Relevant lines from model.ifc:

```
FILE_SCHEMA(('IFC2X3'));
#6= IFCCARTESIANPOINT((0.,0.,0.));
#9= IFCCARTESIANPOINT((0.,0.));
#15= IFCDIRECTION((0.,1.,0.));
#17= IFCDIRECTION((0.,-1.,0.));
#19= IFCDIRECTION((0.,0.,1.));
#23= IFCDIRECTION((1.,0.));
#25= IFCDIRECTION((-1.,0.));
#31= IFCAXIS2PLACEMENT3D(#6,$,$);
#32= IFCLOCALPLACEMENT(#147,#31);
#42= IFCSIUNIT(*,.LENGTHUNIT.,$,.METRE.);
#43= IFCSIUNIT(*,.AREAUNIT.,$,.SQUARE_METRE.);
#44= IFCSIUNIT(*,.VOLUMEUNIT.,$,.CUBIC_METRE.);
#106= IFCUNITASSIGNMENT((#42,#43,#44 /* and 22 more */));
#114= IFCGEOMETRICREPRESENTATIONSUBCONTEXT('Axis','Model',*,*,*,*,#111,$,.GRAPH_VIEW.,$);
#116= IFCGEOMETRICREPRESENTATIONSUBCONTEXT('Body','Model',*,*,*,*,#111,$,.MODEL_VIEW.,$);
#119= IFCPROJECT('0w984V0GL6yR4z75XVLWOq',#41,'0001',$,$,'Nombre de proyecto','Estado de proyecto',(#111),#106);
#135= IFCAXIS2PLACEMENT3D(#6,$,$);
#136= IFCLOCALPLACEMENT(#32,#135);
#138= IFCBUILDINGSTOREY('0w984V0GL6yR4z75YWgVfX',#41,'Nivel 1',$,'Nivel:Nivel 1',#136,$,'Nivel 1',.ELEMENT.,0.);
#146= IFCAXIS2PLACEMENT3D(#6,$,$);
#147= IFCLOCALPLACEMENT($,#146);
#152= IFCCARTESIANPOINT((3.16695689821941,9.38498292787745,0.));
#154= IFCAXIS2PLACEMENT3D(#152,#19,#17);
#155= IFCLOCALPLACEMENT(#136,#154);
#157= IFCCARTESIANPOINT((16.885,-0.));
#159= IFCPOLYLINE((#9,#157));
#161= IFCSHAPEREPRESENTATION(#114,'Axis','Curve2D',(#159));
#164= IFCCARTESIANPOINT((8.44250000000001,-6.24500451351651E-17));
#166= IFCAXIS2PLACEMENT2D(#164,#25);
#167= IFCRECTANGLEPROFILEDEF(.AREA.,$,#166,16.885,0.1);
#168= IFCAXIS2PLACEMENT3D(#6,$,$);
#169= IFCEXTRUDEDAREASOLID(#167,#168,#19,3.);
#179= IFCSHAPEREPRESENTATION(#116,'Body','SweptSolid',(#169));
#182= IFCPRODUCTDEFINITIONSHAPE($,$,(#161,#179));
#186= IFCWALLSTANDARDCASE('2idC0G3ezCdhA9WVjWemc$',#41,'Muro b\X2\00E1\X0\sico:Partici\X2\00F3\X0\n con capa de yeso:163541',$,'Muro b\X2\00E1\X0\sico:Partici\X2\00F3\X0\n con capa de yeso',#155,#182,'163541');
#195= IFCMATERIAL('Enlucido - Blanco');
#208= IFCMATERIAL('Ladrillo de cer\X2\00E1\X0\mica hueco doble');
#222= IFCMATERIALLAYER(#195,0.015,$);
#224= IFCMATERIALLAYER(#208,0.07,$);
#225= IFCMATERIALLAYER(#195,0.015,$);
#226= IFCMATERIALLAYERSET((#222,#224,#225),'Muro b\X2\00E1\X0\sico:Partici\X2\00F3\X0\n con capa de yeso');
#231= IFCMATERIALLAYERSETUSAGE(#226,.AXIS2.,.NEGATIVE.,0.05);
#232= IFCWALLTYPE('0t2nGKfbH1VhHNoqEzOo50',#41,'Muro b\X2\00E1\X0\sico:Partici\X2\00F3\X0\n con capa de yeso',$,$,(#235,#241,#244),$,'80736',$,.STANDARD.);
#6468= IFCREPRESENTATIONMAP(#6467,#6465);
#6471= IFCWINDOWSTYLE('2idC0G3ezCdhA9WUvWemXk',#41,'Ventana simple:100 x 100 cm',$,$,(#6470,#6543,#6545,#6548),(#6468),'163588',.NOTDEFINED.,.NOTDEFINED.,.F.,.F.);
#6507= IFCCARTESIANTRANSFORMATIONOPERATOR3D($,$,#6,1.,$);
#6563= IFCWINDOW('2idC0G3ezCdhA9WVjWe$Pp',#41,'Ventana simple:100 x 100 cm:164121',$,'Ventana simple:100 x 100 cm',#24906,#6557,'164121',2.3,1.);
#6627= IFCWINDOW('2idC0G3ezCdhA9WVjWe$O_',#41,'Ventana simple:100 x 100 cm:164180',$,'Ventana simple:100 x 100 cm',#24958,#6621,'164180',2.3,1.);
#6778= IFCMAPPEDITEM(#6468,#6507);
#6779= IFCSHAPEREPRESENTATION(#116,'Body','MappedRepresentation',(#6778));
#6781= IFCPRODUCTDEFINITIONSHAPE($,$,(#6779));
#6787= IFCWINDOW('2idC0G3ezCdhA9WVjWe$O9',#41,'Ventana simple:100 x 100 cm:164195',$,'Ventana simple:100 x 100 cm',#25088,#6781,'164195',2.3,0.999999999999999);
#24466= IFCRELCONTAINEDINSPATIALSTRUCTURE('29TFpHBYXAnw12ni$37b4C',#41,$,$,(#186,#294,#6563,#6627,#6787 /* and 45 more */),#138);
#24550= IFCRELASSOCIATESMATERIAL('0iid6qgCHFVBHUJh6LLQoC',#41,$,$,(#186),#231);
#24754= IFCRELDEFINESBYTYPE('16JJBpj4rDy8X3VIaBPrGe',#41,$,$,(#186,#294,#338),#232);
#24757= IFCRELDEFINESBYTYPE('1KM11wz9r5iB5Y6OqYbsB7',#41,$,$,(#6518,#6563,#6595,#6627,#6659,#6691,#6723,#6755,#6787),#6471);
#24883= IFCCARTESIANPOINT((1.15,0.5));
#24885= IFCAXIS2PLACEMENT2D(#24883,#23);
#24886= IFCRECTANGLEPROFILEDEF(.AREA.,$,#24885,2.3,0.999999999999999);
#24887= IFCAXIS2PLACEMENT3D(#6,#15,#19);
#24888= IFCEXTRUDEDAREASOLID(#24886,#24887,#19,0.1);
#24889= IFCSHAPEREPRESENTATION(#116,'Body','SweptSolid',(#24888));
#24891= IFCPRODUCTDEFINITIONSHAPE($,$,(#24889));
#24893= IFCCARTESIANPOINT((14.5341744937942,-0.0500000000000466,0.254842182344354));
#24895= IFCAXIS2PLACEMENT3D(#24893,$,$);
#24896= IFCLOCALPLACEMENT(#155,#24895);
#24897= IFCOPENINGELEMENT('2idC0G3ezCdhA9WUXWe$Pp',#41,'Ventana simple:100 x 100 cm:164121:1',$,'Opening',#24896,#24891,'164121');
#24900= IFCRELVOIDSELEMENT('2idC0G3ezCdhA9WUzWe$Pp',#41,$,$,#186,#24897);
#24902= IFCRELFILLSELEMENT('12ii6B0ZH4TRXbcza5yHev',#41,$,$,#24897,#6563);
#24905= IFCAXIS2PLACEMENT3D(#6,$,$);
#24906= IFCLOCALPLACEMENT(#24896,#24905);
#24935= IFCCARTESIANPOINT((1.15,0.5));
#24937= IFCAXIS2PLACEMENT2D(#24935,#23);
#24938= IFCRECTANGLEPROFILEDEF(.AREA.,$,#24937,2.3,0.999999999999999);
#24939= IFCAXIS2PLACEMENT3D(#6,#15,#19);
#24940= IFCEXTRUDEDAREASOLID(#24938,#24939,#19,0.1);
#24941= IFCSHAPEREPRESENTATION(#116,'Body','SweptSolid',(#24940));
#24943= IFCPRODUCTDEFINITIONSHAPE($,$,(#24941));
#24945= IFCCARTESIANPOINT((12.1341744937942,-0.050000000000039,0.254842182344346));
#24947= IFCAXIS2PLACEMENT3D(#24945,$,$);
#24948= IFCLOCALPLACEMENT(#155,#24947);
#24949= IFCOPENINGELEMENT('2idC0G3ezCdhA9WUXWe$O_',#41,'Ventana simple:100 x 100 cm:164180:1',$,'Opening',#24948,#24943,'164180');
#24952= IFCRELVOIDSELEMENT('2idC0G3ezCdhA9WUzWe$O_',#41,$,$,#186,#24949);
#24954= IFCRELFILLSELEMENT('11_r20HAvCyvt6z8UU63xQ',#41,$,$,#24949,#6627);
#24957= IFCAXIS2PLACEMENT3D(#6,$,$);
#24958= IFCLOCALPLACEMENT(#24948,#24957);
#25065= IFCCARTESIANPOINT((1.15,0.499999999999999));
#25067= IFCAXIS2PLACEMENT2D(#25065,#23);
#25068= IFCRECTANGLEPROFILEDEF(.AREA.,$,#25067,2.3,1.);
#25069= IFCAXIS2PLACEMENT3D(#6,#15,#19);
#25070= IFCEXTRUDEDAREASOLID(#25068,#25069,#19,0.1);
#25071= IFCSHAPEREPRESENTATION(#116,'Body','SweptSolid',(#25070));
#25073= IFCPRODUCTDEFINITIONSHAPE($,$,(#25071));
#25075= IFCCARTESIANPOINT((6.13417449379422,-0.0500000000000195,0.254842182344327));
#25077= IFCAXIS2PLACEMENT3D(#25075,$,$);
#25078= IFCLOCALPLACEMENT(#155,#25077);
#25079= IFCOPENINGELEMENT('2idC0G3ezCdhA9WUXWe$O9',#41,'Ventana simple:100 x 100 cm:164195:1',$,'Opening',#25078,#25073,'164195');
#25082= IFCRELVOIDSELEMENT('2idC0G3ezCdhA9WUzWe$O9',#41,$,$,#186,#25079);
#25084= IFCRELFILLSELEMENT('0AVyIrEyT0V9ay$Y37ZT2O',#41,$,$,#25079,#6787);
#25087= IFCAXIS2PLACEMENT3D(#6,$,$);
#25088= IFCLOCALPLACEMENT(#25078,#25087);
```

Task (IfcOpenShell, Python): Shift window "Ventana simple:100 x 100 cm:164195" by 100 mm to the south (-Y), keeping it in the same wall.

```python
import ifcopenshell
import ifcopenshell.api.geometry
import ifcopenshell.util.placement

model = ifcopenshell.open("model.ifc")

window = model.by_id(6787)
opening = window.FillsVoids[0].RelatingOpeningElement
wall = opening.VoidsElements[0].RelatingBuildingElement

wall_matrix = ifcopenshell.util.placement.get_local_placement(wall.ObjectPlacement)
shift = wall_matrix[:3, 0] * 0.1
before = ifcopenshell.util.placement.get_local_placement(window.ObjectPlacement)[:3, 3].copy()

# The window is placed relative to its opening, so it follows when the opening moves.
matrix = ifcopenshell.util.placement.get_local_placement(opening.ObjectPlacement)
matrix[:3, 3] += shift
ifcopenshell.api.geometry.edit_object_placement(
    model, product=opening, matrix=matrix, is_si=False, should_transform_children=True
)

after = ifcopenshell.util.placement.get_local_placement(window.ObjectPlacement)[:3, 3]
print("window moved by", (after - before).round(3) + 0.0)

model.write("model_updated.ifc")
```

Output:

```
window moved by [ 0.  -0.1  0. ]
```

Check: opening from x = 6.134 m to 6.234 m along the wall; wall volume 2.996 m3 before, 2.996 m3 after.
